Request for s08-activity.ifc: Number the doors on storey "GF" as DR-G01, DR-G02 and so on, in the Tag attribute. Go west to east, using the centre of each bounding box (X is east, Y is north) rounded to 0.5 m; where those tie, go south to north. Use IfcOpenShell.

First a look at what the model holds.

```python
import ifcopenshell
import ifcopenshell.util.element
import ifcopenshell.util.placement

model = ifcopenshell.open("s08-activity.ifc")
print(model.schema)
storey = next(s for s in model.by_type("IfcBuildingStorey") if s.Name == "GF")
doors = [e for e in ifcopenshell.util.element.get_decomposition(storey) if e.is_a("IfcDoor")]
for e in sorted(doors, key=lambda e: e.id()):
    origin = ifcopenshell.util.placement.get_local_placement(e.ObjectPlacement)[:3, 3]
    print(e.id(), e.Tag, e.Name, origin.round(2) + 0.0, sep=" | ")
```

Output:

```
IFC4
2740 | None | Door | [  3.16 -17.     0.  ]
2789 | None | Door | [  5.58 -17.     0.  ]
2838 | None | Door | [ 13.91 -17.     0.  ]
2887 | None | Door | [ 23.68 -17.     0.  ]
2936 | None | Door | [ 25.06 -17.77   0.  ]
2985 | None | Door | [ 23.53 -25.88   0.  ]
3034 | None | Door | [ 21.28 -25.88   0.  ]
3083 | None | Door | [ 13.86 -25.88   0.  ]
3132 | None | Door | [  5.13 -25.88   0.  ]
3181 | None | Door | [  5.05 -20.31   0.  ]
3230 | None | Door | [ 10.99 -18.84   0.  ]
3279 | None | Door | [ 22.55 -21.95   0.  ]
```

```python
import ifcopenshell
import ifcopenshell.geom
import ifcopenshell.util.element
import ifcopenshell.util.shape

model = ifcopenshell.open("s08-activity.ifc")
settings = ifcopenshell.geom.settings()
settings.set("use-world-coords", True)


def centre(element):
    shape = ifcopenshell.geom.create_shape(settings, element)
    return ifcopenshell.util.shape.get_bbox_centroid(shape.geometry)


storey = next(s for s in model.by_type("IfcBuildingStorey") if s.Name == "GF")
doors = [e for e in ifcopenshell.util.element.get_decomposition(storey) if e.is_a("IfcDoor")]

# Insertion points can sit at a corner or the storey origin, so sort by the geometry (in metres).
centres = {e: centre(e) for e in doors}
doors.sort(key=lambda e: (round(centres[e][0] / 0.5), centres[e][1]))

for i, e in enumerate(doors, start=1):
    number = f"DR-G{i:02d}"
    e.Tag = number
    print(e.id(), number)

model.write("s08-activity_edited.ifc")
```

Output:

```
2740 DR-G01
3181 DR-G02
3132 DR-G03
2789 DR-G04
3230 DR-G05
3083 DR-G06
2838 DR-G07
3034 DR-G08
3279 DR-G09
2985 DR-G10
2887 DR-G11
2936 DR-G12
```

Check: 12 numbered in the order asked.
